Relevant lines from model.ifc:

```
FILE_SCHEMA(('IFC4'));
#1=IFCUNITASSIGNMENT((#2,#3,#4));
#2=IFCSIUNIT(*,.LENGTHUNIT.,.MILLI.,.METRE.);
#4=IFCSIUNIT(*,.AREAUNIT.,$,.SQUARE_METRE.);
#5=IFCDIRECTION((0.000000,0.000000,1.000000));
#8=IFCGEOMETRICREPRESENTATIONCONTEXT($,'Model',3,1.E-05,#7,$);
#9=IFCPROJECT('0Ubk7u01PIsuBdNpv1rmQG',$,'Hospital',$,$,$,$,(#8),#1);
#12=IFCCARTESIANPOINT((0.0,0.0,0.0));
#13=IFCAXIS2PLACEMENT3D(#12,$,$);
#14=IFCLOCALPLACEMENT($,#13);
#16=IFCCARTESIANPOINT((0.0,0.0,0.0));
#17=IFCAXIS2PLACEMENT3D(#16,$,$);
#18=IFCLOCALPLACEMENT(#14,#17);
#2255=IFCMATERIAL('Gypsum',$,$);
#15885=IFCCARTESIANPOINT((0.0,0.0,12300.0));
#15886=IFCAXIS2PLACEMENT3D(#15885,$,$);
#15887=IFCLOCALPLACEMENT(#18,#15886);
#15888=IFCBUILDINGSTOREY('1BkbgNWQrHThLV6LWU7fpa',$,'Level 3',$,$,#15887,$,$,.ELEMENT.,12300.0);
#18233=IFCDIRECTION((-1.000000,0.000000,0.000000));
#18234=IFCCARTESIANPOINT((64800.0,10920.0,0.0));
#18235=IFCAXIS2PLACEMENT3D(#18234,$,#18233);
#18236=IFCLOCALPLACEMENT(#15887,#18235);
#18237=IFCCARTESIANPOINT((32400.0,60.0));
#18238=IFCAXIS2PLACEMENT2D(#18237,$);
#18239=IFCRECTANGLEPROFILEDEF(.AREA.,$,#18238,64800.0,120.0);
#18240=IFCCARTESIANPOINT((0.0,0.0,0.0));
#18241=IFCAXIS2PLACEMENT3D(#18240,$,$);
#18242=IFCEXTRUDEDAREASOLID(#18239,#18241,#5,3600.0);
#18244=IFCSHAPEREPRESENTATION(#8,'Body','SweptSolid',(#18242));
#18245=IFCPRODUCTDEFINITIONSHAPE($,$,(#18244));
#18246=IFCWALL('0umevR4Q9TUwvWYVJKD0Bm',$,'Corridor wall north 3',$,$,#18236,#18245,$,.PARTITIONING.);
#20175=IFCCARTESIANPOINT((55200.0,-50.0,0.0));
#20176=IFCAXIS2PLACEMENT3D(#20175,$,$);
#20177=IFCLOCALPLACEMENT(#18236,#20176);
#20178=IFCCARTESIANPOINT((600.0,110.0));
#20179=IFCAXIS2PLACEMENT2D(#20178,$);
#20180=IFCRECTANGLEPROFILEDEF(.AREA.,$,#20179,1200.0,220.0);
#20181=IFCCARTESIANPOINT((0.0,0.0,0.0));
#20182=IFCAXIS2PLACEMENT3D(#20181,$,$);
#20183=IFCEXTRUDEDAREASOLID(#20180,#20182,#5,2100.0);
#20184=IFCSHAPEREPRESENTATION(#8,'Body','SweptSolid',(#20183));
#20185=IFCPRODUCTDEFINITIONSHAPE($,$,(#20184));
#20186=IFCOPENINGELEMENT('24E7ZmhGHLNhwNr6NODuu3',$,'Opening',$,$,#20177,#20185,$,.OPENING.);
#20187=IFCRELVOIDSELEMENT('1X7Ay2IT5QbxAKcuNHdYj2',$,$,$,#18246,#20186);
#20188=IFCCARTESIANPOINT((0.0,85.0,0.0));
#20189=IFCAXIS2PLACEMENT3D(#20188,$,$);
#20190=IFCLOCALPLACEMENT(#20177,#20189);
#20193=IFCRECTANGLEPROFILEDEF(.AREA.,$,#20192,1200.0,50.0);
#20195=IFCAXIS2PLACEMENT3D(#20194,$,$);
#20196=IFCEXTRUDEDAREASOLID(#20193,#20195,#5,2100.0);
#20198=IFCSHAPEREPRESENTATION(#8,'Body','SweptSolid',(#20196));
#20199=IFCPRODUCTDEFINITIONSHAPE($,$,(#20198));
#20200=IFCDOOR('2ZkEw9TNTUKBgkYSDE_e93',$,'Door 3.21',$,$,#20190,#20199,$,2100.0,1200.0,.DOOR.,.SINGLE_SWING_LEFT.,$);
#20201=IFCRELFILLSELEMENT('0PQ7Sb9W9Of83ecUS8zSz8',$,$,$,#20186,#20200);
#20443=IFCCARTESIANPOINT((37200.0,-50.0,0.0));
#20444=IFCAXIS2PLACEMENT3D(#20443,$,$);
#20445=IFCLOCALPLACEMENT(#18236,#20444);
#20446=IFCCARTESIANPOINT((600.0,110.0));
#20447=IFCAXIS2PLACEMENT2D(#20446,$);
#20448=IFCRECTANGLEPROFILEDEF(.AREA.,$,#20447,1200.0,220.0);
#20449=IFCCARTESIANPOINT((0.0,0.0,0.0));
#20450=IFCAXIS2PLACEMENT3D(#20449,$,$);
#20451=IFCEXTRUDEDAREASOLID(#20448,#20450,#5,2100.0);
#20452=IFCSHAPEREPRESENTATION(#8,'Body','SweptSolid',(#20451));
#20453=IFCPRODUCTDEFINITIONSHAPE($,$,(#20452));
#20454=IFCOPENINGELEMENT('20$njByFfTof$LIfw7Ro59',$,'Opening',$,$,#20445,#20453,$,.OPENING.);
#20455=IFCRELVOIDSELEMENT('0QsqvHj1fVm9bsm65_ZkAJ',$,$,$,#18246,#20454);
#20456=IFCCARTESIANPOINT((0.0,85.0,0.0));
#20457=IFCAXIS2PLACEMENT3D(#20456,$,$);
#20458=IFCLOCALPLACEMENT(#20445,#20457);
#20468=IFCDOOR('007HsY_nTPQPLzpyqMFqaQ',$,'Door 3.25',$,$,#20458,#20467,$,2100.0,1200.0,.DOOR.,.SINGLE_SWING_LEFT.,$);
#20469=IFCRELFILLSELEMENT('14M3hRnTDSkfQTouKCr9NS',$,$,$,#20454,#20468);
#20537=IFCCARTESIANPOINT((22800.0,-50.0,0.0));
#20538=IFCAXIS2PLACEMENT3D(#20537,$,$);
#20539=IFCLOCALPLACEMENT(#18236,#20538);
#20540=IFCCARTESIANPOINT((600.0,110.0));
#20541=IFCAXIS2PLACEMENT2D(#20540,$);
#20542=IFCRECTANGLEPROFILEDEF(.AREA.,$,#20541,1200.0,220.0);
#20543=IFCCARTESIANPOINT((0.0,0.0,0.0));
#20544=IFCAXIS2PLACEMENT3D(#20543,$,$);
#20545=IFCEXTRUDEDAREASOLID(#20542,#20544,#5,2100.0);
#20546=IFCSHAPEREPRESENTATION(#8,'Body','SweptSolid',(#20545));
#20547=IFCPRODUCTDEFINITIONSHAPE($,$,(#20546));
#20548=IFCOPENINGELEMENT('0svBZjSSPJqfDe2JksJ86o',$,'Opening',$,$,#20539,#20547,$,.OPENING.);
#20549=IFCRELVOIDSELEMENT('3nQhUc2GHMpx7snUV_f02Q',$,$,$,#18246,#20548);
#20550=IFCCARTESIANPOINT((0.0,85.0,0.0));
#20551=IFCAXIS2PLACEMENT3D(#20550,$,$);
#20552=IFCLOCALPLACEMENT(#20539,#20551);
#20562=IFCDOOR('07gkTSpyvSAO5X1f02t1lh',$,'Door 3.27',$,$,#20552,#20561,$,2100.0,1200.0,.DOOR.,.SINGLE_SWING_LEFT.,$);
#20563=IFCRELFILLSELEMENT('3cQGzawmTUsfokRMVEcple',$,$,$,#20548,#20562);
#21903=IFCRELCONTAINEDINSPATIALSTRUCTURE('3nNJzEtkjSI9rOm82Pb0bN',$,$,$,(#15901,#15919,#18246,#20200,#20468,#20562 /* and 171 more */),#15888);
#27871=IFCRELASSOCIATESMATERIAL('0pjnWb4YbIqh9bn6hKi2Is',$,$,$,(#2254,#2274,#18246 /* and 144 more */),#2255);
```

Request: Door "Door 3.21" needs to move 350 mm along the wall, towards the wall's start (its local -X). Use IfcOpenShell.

```python
import ifcopenshell
import ifcopenshell.api.geometry
import ifcopenshell.util.placement
import ifcopenshell.util.unit

model = ifcopenshell.open("model.ifc")
unit_scale = ifcopenshell.util.unit.calculate_unit_scale(model)

door = model.by_guid("2ZkEw9TNTUKBgkYSDE_e93")
opening = door.FillsVoids[0].RelatingOpeningElement
wall = opening.VoidsElements[0].RelatingBuildingElement

wall_matrix = ifcopenshell.util.placement.get_local_placement(wall.ObjectPlacement)
shift = wall_matrix[:3, 0] * -0.35 / unit_scale
before = ifcopenshell.util.placement.get_local_placement(door.ObjectPlacement)[:3, 3].copy()

# The door is placed relative to its opening, so it follows when the opening moves.
matrix = ifcopenshell.util.placement.get_local_placement(opening.ObjectPlacement)
matrix[:3, 3] += shift
ifcopenshell.api.geometry.edit_object_placement(
    model, product=opening, matrix=matrix, is_si=False, should_transform_children=True
)

after = ifcopenshell.util.placement.get_local_placement(door.ObjectPlacement)[:3, 3]
print("door moved by", (after - before).round(3) + 0.0)

model.write("model_updated.ifc")
```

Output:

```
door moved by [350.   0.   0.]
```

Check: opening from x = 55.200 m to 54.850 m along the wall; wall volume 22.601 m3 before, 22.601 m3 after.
